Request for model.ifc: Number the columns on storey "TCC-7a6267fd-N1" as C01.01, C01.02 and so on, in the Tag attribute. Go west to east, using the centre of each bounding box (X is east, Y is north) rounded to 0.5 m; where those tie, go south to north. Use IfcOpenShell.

First a look at what the model holds.

```python
import ifcopenshell
import ifcopenshell.util.element
import ifcopenshell.util.placement

model = ifcopenshell.open("model.ifc")
print(model.schema)
storey = next(s for s in model.by_type("IfcBuildingStorey") if s.Name == "TCC-7a6267fd-N1")
columns = [e for e in ifcopenshell.util.element.get_decomposition(storey) if e.is_a("IfcColumn")]
for e in sorted(columns, key=lambda e: e.id()):
    origin = ifcopenshell.util.placement.get_local_placement(e.ObjectPlacement)[:3, 3]
    print(e.id(), e.Tag, e.Name, origin.round(2) + 0.0, sep=" | ")
```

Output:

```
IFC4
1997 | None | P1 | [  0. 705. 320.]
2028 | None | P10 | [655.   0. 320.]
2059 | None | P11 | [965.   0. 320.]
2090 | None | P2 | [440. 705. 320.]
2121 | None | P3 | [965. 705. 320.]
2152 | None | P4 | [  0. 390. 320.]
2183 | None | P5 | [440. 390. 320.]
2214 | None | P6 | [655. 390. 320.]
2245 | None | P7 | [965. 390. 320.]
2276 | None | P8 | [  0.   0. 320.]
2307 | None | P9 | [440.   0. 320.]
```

```python
import ifcopenshell
import ifcopenshell.geom
import ifcopenshell.util.element
import ifcopenshell.util.shape

model = ifcopenshell.open("model.ifc")
settings = ifcopenshell.geom.settings()
settings.set("use-world-coords", True)


def centre(element):
    shape = ifcopenshell.geom.create_shape(settings, element)
    return ifcopenshell.util.shape.get_bbox_centroid(shape.geometry)


storey = next(s for s in model.by_type("IfcBuildingStorey") if s.Name == "TCC-7a6267fd-N1")
columns = [e for e in ifcopenshell.util.element.get_decomposition(storey) if e.is_a("IfcColumn")]

# Insertion points can sit at a corner or the storey origin, so sort by the geometry (in metres).
centres = {e: centre(e) for e in columns}
columns.sort(key=lambda e: (round(centres[e][0] / 0.5), centres[e][1]))

for i, e in enumerate(columns, start=1):
    number = f"C01.{i:02d}"
    e.Tag = number
    print(e.id(), number)

model.write("model_v2.ifc")
```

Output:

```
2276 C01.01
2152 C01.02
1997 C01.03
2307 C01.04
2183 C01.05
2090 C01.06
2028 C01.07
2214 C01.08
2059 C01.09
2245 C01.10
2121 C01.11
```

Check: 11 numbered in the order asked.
